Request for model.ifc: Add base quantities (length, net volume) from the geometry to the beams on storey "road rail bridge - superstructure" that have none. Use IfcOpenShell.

First a look at what the model holds.

```python
import ifcopenshell
import ifcopenshell.util.element
import ifcopenshell.util.unit

model = ifcopenshell.open("model.ifc")
print(model.schema)
for unit_type in ("LENGTHUNIT", "AREAUNIT", "VOLUMEUNIT"):
    print(unit_type, ifcopenshell.util.unit.calculate_unit_scale(model, unit_type))
storey = next(s for s in model.by_type("IfcBuildingStorey") if s.Name == "road rail bridge - superstructure")
beams = [e for e in ifcopenshell.util.element.get_decomposition(storey) if e.is_a("IfcBeam")]
for e in sorted(beams, key=lambda e: e.id()):
    print(e.id(), e.is_a(), e.Name, list(ifcopenshell.util.element.get_psets(e, qtos_only=True)), sep=" | ")
```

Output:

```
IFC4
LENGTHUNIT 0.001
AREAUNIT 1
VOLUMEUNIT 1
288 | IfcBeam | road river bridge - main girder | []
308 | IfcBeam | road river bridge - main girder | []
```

```python
import ifcopenshell
import ifcopenshell.api.pset
import ifcopenshell.geom
import ifcopenshell.util.element
import ifcopenshell.util.shape
import ifcopenshell.util.unit

model = ifcopenshell.open("model.ifc")
unit_scale = ifcopenshell.util.unit.calculate_unit_scale(model)
volume_scale = ifcopenshell.util.unit.calculate_unit_scale(model, "VOLUMEUNIT")
settings = ifcopenshell.geom.settings()

storey = next(s for s in model.by_type("IfcBuildingStorey") if s.Name == "road rail bridge - superstructure")
beams = [e for e in ifcopenshell.util.element.get_decomposition(storey) if e.is_a("IfcBeam")]

for e in sorted(beams, key=lambda e: e.id()):
    if ifcopenshell.util.element.get_psets(e, qtos_only=True, should_inherit=False):
        continue
    # Geometry comes back in metres, in the element's own axes.
    shape = ifcopenshell.geom.create_shape(settings, e)
    values = {
        "Length": ifcopenshell.util.shape.get_max_xyz(shape.geometry) / unit_scale,
        "NetVolume": ifcopenshell.util.shape.get_volume(shape.geometry) / volume_scale,
    }
    qto = ifcopenshell.api.pset.add_qto(model, product=e, name="Qto_BeamBaseQuantities")
    ifcopenshell.api.pset.edit_qto(model, qto=qto, properties=values)
    print(e.id(), {k: round(v, 3) for k, v in values.items()})

model.write("model_updated.ifc")
```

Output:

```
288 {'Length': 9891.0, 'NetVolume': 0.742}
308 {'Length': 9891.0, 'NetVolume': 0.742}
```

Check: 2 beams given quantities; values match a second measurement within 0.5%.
